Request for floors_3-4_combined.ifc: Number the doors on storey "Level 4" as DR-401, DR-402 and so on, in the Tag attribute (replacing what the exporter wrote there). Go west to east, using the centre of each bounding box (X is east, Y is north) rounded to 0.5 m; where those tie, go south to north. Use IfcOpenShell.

First a look at what the model holds.

```python
import ifcopenshell
import ifcopenshell.util.element
import ifcopenshell.util.placement

model = ifcopenshell.open("floors_3-4_combined.ifc")
print(model.schema)
storey = next(s for s in model.by_type("IfcBuildingStorey") if s.Name == "Level 4")
doors = [e for e in ifcopenshell.util.element.get_decomposition(storey) if e.is_a("IfcDoor")]
for e in sorted(doors, key=lambda e: e.id()):
    origin = ifcopenshell.util.placement.get_local_placement(e.ObjectPlacement)[:3, 3]
    print(e.id(), e.Tag, e.Name, origin.round(2) + 0.0, sep=" | ")
```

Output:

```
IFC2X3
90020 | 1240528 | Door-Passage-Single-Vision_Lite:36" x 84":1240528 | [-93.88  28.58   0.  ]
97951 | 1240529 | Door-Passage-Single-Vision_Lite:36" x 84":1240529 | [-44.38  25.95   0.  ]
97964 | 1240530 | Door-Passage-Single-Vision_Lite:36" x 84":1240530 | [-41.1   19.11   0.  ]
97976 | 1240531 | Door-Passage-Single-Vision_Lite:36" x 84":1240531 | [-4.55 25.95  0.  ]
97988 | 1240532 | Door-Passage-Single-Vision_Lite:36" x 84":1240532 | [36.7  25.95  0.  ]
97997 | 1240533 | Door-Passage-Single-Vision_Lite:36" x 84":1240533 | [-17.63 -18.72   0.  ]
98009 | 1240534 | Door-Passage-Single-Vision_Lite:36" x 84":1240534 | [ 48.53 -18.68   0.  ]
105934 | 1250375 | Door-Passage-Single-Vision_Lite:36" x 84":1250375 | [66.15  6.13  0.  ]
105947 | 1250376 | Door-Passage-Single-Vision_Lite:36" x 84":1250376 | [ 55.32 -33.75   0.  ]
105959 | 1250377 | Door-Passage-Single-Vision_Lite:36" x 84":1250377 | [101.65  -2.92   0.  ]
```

```python
import ifcopenshell
import ifcopenshell.geom
import ifcopenshell.util.element
import ifcopenshell.util.shape

model = ifcopenshell.open("floors_3-4_combined.ifc")
settings = ifcopenshell.geom.settings()
settings.set("use-world-coords", True)


def centre(element):
    shape = ifcopenshell.geom.create_shape(settings, element)
    return ifcopenshell.util.shape.get_bbox_centroid(shape.geometry)


storey = next(s for s in model.by_type("IfcBuildingStorey") if s.Name == "Level 4")
doors = [e for e in ifcopenshell.util.element.get_decomposition(storey) if e.is_a("IfcDoor")]

# Insertion points can sit at a corner or the storey origin, so sort by the geometry (in metres).
centres = {e: centre(e) for e in doors}
doors.sort(key=lambda e: (round(centres[e][0] / 0.5), centres[e][1]))

for i, e in enumerate(doors, start=1):
    number = f"DR-4{i:02d}"
    e.Tag = number
    print(e.id(), number)

model.write("floors_3-4_combined_rev.ifc")
```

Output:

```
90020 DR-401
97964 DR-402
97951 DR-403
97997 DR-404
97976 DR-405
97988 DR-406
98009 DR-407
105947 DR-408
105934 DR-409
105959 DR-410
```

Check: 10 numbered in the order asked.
